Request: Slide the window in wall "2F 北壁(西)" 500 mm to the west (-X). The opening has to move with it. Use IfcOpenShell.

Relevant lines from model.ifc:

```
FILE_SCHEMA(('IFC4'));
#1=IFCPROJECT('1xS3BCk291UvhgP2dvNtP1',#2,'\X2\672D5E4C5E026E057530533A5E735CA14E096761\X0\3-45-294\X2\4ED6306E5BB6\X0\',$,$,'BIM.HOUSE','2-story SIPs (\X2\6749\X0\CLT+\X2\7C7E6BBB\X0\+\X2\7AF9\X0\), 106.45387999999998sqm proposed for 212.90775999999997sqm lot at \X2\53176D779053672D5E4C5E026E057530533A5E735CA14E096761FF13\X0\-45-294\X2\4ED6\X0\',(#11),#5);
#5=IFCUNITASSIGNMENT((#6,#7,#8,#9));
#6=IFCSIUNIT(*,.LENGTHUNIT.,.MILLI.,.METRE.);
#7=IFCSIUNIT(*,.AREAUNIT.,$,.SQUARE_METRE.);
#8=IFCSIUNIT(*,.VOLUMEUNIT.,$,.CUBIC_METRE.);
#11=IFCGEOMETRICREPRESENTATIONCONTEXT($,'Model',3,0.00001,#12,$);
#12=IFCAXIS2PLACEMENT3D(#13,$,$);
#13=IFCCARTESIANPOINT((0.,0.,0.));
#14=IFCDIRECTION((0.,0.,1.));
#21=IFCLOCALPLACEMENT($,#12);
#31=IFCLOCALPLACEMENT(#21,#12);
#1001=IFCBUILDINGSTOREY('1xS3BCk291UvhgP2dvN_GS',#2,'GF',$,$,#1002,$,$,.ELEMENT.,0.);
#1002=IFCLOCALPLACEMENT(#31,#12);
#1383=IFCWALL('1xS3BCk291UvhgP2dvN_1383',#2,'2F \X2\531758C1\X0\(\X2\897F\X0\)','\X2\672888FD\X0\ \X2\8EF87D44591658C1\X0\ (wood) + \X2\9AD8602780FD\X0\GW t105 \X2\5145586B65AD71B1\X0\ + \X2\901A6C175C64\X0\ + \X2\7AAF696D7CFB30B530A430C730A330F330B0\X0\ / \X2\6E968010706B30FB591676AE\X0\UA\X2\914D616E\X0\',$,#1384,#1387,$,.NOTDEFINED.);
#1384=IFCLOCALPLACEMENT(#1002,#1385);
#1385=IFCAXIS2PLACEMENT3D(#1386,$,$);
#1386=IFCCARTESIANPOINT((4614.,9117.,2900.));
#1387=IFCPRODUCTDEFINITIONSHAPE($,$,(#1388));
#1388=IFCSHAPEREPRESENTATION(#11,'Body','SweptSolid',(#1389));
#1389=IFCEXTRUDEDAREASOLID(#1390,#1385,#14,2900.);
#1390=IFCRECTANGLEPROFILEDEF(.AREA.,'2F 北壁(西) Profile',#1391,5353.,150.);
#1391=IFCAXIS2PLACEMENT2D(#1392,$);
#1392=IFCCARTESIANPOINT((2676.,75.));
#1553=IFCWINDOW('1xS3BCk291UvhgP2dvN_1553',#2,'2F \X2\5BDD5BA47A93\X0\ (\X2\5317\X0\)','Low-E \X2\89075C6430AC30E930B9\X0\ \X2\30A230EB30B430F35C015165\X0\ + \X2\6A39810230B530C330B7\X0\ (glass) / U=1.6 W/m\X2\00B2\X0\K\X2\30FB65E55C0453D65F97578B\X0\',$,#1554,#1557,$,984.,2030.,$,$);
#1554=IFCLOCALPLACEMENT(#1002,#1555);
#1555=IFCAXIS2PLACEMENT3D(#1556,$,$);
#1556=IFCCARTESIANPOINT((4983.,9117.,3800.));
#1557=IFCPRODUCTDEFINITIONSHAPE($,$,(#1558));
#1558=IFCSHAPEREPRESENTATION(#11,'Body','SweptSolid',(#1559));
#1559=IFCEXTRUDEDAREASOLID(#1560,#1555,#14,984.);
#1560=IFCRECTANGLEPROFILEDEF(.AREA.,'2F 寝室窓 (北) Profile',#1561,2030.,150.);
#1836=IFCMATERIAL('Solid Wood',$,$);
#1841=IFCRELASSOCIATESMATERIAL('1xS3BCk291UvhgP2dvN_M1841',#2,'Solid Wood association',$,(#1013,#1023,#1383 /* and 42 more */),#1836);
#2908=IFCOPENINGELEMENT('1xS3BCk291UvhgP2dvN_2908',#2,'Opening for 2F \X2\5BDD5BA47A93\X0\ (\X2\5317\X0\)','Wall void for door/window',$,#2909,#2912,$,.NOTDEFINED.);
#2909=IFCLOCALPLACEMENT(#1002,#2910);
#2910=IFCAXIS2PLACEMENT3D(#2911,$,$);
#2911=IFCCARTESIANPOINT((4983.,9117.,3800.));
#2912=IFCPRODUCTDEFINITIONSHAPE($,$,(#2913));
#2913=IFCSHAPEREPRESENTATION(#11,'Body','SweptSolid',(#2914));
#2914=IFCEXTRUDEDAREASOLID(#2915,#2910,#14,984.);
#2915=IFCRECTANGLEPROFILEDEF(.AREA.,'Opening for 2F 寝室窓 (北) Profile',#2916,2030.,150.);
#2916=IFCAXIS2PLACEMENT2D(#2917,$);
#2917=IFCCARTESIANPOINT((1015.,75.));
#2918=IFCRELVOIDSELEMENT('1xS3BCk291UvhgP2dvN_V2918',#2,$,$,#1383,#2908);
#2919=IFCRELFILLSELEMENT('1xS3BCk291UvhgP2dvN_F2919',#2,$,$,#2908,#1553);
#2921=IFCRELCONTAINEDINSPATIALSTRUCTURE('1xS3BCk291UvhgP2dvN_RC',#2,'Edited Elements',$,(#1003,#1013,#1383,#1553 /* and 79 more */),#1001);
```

```python
import ifcopenshell
import ifcopenshell.api.geometry
import ifcopenshell.util.placement
import ifcopenshell.util.unit

model = ifcopenshell.open("model.ifc")
unit_scale = ifcopenshell.util.unit.calculate_unit_scale(model)

window = model.by_guid("1xS3BCk291UvhgP2dvN_1553")
opening = window.FillsVoids[0].RelatingOpeningElement
wall = opening.VoidsElements[0].RelatingBuildingElement

wall_matrix = ifcopenshell.util.placement.get_local_placement(wall.ObjectPlacement)
shift = wall_matrix[:3, 0] * -0.5 / unit_scale
before = ifcopenshell.util.placement.get_local_placement(window.ObjectPlacement)[:3, 3].copy()

# The window is not placed relative to its opening, so move both.
for product in (opening, window):
    matrix = ifcopenshell.util.placement.get_local_placement(product.ObjectPlacement)
    matrix[:3, 3] += shift
    ifcopenshell.api.geometry.edit_object_placement(model, product=product, matrix=matrix, is_si=False)

after = ifcopenshell.util.placement.get_local_placement(window.ObjectPlacement)[:3, 3]
print("window moved by", (after - before).round(3) + 0.0)

model.write("model_rev.ifc")
```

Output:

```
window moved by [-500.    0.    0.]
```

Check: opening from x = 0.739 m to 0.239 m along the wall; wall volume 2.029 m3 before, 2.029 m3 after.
